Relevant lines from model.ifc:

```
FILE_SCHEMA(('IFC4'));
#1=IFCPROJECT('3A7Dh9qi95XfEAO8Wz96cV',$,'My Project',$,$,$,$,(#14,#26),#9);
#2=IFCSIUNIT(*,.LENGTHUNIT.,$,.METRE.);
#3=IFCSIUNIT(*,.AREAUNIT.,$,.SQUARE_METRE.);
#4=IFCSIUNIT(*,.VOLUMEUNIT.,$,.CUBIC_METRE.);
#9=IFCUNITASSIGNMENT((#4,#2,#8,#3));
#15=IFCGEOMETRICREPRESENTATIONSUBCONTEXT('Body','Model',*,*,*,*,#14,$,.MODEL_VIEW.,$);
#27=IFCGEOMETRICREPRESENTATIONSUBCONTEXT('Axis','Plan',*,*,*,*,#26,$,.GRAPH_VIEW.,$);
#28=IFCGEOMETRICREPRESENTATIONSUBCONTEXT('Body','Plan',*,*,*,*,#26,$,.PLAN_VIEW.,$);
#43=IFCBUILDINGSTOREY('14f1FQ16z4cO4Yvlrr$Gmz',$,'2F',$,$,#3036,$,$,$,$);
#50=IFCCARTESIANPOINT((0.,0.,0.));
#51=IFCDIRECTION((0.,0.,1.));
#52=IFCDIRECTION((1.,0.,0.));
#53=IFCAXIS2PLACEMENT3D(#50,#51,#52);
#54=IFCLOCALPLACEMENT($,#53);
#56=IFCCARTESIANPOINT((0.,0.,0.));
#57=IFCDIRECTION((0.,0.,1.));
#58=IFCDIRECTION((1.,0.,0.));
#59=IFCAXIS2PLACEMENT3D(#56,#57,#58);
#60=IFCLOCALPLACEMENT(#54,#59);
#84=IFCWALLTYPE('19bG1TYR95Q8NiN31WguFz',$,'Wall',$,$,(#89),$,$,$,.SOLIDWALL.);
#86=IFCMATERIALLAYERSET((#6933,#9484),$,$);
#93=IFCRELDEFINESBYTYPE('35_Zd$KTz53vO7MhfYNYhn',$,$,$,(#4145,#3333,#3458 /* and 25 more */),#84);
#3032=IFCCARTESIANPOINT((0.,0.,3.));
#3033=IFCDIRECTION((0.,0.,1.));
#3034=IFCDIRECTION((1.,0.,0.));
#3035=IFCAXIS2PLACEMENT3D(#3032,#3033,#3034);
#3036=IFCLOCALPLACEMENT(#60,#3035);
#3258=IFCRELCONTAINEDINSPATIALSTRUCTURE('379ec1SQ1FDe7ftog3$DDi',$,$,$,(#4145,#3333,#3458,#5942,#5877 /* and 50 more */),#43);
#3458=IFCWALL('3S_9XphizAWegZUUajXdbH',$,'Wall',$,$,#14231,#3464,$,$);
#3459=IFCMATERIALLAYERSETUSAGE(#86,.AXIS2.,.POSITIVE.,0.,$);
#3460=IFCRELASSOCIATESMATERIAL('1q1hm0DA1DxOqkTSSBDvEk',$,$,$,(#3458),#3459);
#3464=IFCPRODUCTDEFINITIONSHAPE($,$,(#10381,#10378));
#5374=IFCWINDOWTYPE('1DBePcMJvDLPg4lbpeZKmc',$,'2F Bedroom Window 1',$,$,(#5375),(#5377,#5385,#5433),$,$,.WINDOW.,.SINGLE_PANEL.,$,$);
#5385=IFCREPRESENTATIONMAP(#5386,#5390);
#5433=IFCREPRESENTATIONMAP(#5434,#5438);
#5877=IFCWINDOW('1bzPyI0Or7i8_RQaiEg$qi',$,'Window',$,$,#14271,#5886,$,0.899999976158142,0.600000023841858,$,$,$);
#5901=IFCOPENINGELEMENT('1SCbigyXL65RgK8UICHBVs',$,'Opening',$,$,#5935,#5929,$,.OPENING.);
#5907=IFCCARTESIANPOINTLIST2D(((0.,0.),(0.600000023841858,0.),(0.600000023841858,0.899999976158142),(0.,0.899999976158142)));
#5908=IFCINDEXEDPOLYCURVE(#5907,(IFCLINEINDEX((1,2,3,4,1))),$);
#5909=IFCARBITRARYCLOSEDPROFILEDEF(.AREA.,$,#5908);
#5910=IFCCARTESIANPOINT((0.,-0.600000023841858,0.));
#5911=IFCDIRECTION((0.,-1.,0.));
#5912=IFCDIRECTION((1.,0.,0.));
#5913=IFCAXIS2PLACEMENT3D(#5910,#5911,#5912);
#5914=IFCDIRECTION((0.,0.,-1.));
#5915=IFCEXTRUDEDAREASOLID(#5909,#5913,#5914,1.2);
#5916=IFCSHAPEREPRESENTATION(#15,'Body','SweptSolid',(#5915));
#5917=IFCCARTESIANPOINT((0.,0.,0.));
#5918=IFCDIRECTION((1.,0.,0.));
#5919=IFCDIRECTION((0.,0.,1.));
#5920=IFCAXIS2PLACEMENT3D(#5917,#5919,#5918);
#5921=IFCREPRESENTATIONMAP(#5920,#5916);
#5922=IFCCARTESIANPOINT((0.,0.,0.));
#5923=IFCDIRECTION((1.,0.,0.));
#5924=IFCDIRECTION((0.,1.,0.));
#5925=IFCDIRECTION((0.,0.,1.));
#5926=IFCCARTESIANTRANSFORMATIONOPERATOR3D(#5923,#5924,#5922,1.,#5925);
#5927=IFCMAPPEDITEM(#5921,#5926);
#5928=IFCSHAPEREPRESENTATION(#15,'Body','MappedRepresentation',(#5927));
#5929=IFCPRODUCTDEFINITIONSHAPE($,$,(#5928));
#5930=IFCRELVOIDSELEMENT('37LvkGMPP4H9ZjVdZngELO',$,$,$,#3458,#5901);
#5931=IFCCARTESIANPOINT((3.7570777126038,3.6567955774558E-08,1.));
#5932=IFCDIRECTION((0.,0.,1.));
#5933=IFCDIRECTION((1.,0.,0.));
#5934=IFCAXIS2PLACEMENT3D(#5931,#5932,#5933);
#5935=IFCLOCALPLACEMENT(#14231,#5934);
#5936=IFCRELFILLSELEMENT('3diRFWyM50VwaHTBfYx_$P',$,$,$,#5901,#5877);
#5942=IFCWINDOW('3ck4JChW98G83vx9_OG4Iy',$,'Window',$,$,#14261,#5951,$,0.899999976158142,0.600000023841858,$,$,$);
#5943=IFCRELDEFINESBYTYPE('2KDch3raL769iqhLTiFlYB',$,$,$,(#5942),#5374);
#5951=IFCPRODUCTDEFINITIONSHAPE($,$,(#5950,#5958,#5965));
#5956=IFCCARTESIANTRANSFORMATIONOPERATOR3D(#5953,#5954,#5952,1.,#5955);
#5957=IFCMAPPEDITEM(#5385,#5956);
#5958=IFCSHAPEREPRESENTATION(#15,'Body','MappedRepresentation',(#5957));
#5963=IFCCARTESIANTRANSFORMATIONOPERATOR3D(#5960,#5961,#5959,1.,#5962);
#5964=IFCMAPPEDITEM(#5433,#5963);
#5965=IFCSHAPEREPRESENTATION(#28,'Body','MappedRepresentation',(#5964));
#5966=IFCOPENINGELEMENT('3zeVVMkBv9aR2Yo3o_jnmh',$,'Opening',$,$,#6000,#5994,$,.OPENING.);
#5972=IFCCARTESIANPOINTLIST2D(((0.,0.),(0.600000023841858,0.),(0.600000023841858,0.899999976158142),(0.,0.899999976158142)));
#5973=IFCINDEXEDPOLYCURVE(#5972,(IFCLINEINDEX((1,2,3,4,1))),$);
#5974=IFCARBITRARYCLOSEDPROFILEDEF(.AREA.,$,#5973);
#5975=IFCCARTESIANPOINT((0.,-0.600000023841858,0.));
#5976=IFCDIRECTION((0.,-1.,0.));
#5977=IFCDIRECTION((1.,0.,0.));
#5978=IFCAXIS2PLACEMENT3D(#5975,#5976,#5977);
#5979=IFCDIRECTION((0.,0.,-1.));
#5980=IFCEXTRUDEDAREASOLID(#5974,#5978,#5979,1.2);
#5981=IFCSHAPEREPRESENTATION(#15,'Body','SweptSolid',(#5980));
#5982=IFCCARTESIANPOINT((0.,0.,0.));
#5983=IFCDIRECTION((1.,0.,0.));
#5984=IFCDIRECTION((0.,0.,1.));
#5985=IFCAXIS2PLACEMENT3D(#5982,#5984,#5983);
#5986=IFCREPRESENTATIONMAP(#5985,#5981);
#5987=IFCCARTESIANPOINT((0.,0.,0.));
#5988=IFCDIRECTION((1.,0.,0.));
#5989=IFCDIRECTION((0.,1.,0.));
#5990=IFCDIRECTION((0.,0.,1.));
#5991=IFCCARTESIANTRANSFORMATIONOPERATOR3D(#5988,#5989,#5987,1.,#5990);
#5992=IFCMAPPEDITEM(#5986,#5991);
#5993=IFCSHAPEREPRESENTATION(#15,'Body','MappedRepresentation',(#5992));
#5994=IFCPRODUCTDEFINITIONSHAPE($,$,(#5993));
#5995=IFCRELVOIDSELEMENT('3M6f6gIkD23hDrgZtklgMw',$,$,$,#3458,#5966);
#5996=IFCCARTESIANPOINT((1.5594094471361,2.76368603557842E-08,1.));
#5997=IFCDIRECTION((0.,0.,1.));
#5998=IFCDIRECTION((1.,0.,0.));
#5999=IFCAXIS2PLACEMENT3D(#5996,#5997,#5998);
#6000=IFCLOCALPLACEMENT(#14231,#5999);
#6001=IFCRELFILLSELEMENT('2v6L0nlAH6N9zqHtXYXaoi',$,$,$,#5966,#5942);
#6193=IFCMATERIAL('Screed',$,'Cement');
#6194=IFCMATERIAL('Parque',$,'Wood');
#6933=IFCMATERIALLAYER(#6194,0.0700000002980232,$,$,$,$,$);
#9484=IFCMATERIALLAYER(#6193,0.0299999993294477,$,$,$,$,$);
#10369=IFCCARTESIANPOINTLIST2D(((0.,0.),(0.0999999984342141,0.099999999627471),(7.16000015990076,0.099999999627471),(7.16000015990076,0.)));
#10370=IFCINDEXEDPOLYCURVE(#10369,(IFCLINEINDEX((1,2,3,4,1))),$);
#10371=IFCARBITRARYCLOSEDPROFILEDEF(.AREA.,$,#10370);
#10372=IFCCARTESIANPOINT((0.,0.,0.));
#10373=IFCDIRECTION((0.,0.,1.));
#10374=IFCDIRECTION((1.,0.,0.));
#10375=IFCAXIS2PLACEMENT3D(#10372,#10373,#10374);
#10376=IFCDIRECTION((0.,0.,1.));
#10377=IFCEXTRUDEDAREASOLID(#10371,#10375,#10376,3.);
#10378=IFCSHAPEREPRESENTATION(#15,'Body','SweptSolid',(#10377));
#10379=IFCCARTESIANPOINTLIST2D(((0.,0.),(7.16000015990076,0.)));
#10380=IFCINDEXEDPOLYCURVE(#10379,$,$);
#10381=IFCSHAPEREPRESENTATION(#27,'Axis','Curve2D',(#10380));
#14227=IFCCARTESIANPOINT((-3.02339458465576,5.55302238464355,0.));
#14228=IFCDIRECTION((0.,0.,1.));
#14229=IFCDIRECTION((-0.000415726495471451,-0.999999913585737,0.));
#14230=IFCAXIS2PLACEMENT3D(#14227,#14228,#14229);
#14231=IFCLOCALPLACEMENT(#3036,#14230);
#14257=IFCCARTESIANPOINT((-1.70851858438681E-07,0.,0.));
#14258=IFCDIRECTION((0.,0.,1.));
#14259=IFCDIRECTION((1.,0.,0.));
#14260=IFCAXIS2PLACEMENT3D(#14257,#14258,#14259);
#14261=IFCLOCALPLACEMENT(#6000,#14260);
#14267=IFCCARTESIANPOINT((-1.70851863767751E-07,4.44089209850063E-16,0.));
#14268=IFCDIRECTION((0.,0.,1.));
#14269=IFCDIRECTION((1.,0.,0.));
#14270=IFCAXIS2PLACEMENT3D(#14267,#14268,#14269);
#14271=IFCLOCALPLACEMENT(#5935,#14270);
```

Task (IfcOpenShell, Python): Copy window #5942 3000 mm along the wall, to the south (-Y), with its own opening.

```python
import ifcopenshell
import ifcopenshell.api.feature
import ifcopenshell.api.geometry
import ifcopenshell.api.root
import ifcopenshell.geom
import ifcopenshell.util.element
import ifcopenshell.util.placement
import ifcopenshell.util.shape
import ifcopenshell.util.unit

model = ifcopenshell.open("model.ifc")
unit_scale = ifcopenshell.util.unit.calculate_unit_scale(model)
settings = ifcopenshell.geom.settings()


def volume(element):
    """Net volume in cubic metres, openings subtracted."""
    shape = ifcopenshell.geom.create_shape(settings, element)
    return ifcopenshell.util.shape.get_volume(shape.geometry)


window = model.by_guid("3ck4JChW98G83vx9_OG4Iy")
opening = window.FillsVoids[0].RelatingOpeningElement
wall = opening.VoidsElements[0].RelatingBuildingElement
before = volume(wall)
shift = ifcopenshell.util.placement.get_local_placement(wall.ObjectPlacement)[:3, 0] * 3 / unit_scale

# copy_class copies the void relationship, type, container and properties, but no geometry.
new_opening = ifcopenshell.api.root.copy_class(model, product=opening)
new_opening.Representation = ifcopenshell.util.element.copy_deep(
    model, opening.Representation, exclude=["IfcGeometricRepresentationContext", "IfcRepresentationMap"]
)
new_window = ifcopenshell.api.root.copy_class(model, product=window)
new_window.Representation = ifcopenshell.util.element.copy_deep(
    model, window.Representation, exclude=["IfcGeometricRepresentationContext", "IfcRepresentationMap"]
)
ifcopenshell.api.feature.add_filling(model, opening=new_opening, element=new_window)

for old, new in ((opening, new_opening), (window, new_window)):
    matrix = ifcopenshell.util.placement.get_local_placement(old.ObjectPlacement)
    matrix[:3, 3] += shift
    ifcopenshell.api.geometry.edit_object_placement(model, product=new, matrix=matrix, is_si=False)

after = volume(wall)

print(f"wall volume {before:.3f} -> {after:.3f} m3")

model.write("model_edited.ifc")
```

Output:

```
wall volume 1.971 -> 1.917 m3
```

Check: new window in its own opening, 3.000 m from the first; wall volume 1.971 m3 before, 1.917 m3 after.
